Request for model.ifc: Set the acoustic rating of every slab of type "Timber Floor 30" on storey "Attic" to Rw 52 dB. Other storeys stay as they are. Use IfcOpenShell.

First a look at what the model holds.

```python
import ifcopenshell
import ifcopenshell.util.element

model = ifcopenshell.open("model.ifc")
print(model.schema)
storey = next(s for s in model.by_type("IfcBuildingStorey") if s.Name == "Attic")
slabs = [e for e in ifcopenshell.util.element.get_decomposition(storey) if e.is_a("IfcSlab")]
seen = {}
for e in slabs:
    element_type = ifcopenshell.util.element.get_type(e)
    key = (element_type.Name if element_type != e and element_type else None, ifcopenshell.util.element.get_pset(e, "Pset_SlabCommon", "AcousticRating"))
    seen[key] = seen.get(key, 0) + 1
for (name, value), count in sorted(seen.items(), key=str):
    print(count, "x", name, "|", value)
```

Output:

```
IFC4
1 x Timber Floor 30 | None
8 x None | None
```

```python
import ifcopenshell
import ifcopenshell.api.pset
import ifcopenshell.util.element

model = ifcopenshell.open("model.ifc")

storey = next(s for s in model.by_type("IfcBuildingStorey") if s.Name == "Attic")
slabs = [e for e in ifcopenshell.util.element.get_decomposition(storey) if e.is_a("IfcSlab")]

count = 0
for e in slabs:
    element_type = ifcopenshell.util.element.get_type(e)
    if element_type in (None, e) or element_type.Name != "Timber Floor 30":
        continue
    # add_pset returns the element's existing set when there is one.
    pset = ifcopenshell.api.pset.add_pset(model, product=e, name="Pset_SlabCommon")
    ifcopenshell.api.pset.edit_pset(model, pset=pset, properties={"AcousticRating": "Rw 52 dB"})
    count += 1

print(count, "slabs updated")

model.write("model_v2.ifc")
```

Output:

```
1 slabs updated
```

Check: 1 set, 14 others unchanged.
